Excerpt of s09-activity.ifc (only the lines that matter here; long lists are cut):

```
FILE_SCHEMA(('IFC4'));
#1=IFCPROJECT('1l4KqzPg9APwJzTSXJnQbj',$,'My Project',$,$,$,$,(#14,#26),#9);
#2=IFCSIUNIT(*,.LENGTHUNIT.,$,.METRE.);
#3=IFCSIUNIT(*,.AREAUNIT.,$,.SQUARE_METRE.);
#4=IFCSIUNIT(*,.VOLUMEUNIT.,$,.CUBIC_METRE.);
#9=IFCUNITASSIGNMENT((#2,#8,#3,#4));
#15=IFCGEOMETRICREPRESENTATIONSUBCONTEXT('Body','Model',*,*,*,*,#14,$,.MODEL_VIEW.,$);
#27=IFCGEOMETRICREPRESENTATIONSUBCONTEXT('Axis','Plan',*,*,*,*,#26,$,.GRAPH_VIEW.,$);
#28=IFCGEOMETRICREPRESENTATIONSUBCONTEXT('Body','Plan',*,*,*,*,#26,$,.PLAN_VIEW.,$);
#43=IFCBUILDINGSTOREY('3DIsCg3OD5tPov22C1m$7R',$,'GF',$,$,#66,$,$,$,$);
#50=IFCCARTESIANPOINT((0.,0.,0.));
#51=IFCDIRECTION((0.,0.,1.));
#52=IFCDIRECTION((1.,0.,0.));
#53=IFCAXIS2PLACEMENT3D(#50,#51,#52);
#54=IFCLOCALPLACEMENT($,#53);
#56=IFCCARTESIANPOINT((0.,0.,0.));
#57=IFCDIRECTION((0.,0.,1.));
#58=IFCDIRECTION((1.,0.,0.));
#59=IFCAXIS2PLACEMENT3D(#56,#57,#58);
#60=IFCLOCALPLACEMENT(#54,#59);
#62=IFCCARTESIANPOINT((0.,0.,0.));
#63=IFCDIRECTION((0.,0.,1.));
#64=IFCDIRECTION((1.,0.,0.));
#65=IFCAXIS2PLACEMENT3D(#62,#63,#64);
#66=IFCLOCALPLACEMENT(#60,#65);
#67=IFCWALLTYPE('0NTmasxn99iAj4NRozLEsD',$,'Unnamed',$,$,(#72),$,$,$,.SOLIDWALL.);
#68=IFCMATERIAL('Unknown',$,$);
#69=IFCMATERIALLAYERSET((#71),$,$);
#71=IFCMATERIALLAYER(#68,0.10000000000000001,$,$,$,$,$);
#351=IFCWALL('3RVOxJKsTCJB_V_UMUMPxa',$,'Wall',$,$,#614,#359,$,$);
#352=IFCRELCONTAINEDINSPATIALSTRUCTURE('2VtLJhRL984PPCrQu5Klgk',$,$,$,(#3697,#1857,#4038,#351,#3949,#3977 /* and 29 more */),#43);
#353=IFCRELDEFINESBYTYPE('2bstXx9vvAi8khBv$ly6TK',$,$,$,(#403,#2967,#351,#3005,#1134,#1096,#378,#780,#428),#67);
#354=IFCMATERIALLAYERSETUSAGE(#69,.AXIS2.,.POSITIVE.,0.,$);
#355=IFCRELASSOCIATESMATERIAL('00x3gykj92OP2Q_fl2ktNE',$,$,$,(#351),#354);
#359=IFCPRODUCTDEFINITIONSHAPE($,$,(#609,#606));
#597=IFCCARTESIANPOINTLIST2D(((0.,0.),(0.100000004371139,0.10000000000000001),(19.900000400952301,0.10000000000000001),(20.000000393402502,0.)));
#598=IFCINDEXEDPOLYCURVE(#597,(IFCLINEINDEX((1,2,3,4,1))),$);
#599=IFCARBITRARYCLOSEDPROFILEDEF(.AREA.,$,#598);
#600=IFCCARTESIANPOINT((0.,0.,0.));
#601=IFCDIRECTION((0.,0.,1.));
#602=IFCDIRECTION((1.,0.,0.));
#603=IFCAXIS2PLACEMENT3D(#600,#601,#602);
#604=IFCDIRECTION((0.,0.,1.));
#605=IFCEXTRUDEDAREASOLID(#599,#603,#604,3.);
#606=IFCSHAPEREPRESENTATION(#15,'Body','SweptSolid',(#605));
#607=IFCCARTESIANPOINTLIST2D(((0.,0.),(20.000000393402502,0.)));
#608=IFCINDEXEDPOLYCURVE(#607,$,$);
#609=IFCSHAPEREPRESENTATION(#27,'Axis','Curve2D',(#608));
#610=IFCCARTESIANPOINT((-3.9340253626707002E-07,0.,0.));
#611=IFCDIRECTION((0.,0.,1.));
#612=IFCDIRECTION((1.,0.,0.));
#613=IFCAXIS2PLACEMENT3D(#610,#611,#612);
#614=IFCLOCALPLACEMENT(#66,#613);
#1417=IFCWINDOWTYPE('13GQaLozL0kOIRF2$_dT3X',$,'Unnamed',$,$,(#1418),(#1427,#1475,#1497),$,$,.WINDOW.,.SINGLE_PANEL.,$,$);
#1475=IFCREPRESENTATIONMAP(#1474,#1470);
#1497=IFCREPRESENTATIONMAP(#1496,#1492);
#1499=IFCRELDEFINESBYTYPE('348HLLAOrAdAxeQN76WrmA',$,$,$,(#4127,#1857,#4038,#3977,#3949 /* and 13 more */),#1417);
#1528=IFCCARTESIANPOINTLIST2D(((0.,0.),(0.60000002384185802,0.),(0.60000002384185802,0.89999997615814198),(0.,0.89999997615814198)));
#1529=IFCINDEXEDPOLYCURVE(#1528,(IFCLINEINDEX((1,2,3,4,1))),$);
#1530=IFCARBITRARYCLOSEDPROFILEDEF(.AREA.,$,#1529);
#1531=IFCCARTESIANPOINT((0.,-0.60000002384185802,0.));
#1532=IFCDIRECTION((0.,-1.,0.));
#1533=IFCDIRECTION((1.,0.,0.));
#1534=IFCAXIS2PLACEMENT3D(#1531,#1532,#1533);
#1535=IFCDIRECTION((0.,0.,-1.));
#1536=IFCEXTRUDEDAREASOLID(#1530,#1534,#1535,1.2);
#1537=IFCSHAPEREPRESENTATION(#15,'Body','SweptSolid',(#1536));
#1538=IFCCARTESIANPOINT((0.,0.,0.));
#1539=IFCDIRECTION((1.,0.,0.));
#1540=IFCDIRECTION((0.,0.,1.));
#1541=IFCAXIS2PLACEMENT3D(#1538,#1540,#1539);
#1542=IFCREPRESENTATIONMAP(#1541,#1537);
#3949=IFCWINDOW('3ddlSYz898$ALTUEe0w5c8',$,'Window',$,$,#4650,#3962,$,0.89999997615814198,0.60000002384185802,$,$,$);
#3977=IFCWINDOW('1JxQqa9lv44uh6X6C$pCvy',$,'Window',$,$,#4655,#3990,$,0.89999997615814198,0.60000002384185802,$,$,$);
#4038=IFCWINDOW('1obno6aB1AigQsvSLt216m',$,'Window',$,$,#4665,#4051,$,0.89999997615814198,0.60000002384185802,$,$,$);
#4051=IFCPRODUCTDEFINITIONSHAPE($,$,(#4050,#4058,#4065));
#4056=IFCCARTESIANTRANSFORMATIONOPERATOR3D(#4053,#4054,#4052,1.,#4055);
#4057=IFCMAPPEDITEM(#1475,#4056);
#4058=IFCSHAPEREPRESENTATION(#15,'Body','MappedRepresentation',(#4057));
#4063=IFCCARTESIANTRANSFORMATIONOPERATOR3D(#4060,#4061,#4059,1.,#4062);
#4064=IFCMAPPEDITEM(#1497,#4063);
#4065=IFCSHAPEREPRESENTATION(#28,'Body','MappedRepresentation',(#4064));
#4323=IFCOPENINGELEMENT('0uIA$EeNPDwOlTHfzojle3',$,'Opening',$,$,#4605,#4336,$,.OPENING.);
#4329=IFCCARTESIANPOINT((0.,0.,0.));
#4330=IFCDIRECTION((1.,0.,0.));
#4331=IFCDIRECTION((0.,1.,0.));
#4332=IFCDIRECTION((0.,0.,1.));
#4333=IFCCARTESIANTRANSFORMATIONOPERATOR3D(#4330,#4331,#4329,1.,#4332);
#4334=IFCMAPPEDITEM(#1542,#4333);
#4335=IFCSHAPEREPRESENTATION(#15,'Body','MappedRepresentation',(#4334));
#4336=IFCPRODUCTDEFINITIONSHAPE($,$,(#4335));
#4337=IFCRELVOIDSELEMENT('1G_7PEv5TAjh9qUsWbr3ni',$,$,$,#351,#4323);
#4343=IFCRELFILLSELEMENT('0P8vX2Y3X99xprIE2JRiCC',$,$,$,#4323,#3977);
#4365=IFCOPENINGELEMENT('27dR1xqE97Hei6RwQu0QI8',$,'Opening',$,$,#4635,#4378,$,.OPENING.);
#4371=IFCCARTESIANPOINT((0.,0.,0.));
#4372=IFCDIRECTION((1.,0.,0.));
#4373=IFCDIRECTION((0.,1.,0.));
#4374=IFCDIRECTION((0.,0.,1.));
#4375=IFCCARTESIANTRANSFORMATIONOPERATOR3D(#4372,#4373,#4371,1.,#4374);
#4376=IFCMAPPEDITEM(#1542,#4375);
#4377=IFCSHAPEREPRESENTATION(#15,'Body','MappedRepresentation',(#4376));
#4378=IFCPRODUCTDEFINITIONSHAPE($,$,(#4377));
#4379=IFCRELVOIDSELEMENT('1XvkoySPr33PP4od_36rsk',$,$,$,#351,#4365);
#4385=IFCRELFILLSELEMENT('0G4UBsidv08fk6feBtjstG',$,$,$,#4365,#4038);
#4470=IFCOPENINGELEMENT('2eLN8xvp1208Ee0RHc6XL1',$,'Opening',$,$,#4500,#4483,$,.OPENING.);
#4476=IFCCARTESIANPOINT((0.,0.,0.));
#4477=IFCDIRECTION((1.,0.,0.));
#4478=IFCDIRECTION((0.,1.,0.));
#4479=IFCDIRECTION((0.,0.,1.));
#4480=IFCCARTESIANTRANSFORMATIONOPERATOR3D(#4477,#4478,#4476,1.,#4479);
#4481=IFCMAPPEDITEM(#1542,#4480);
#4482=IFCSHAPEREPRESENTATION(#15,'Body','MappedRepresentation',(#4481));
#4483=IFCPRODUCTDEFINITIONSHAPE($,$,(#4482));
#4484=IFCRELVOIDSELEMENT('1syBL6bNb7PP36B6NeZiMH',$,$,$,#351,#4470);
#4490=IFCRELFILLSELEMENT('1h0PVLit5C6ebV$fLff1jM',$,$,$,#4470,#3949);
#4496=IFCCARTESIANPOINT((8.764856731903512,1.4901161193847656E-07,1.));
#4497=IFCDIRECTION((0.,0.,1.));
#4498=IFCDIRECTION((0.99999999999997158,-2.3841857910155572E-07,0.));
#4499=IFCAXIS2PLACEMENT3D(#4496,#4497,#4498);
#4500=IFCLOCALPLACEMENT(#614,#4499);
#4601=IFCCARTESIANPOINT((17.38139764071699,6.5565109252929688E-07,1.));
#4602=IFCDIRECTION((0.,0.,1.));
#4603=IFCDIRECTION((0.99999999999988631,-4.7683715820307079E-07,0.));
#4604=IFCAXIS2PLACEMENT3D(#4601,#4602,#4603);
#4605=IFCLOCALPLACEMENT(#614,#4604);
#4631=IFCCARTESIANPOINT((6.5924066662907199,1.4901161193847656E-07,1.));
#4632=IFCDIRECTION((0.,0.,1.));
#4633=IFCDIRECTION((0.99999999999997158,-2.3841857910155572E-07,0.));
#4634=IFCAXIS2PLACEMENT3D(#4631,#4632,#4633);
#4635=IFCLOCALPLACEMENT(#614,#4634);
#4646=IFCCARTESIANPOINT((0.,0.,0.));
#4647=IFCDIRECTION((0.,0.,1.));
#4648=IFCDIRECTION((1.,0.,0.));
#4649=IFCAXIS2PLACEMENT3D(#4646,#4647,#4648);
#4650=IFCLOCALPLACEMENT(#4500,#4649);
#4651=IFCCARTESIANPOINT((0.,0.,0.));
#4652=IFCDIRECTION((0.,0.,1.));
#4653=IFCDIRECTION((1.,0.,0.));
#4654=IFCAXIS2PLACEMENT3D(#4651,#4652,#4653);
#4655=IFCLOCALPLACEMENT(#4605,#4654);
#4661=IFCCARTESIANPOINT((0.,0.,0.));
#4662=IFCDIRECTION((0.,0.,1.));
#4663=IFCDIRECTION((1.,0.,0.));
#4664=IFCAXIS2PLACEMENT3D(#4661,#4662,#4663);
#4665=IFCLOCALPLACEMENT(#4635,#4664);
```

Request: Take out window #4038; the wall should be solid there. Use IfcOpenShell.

```python
import ifcopenshell
import ifcopenshell.api.feature
import ifcopenshell.api.root
import ifcopenshell.geom
import ifcopenshell.util.shape

model = ifcopenshell.open("s09-activity.ifc")
settings = ifcopenshell.geom.settings()


def volume(element):
    """Net volume in cubic metres, openings subtracted."""
    shape = ifcopenshell.geom.create_shape(settings, element)
    return ifcopenshell.util.shape.get_volume(shape.geometry)


window = model.by_guid("1obno6aB1AigQsvSLt216m")
opening = window.FillsVoids[0].RelatingOpeningElement
wall = opening.VoidsElements[0].RelatingBuildingElement
before = volume(wall)

ifcopenshell.api.root.remove_product(model, product=window)
ifcopenshell.api.feature.remove_feature(model, feature=opening)

after = volume(wall)

print(f"wall volume {before:.3f} -> {after:.3f} m3")

model.write("s09-activity_updated.ifc")
```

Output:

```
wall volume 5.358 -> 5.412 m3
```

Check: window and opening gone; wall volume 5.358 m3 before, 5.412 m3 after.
